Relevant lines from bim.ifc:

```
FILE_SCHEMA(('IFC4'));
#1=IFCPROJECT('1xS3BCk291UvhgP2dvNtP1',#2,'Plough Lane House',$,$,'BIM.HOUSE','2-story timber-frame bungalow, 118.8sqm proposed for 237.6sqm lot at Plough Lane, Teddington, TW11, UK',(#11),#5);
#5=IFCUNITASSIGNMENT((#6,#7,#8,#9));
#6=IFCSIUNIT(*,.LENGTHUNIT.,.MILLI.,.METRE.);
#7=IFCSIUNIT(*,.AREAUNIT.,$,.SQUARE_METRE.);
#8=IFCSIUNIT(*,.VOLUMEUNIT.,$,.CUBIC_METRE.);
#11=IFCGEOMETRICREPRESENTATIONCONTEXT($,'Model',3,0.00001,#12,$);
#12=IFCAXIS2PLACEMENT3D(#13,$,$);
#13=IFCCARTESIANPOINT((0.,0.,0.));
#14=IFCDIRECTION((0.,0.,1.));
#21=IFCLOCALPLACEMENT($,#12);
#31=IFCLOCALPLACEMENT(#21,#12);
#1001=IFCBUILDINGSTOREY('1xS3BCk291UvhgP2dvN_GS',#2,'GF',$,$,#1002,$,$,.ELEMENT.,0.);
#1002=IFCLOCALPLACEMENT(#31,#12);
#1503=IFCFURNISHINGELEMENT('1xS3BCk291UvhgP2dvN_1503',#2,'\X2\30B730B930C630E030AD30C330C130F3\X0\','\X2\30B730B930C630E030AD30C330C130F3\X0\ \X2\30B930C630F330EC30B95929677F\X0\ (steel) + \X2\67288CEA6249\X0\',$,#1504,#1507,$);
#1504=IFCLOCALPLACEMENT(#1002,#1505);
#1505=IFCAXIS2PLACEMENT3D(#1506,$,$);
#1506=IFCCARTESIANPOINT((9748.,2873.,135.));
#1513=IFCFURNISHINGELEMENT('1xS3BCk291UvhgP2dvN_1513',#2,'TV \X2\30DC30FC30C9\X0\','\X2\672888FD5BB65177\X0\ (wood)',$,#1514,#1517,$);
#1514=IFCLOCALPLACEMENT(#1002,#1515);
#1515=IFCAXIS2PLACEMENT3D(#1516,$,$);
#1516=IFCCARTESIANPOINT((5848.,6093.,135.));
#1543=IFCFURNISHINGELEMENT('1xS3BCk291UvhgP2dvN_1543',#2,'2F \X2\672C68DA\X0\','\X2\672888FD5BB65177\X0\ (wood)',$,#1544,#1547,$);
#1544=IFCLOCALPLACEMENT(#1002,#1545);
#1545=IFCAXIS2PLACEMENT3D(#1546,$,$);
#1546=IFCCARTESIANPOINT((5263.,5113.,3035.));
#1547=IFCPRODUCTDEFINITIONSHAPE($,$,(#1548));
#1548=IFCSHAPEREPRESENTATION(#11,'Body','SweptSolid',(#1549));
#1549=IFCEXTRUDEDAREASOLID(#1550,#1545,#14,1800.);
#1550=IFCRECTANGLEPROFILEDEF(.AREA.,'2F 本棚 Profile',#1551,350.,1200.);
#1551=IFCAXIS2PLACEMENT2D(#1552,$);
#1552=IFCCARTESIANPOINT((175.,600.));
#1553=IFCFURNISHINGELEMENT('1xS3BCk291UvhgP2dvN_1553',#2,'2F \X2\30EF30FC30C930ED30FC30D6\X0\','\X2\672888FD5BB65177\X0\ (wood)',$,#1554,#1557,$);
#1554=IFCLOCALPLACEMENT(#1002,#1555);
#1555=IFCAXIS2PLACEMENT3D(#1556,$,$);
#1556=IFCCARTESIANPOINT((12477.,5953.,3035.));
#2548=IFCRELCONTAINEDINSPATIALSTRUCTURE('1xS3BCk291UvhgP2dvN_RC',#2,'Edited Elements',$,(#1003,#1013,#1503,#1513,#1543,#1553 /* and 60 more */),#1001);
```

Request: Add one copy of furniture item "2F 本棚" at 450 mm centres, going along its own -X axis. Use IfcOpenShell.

```python
import ifcopenshell
import ifcopenshell.api.geometry
import ifcopenshell.api.root
import ifcopenshell.util.element
import ifcopenshell.util.placement

model = ifcopenshell.open("bim.ifc")


def reuse_history(source, copy):
    """copy_class also copies each property set's owner history, people and application; keep the originals."""
    for rel in copy.IsDefinedBy:
        if rel.is_a("IfcRelDefinesByProperties") and (history := rel.RelatingPropertyDefinition.OwnerHistory):
            rel.RelatingPropertyDefinition.OwnerHistory = source.OwnerHistory
            ifcopenshell.util.element.remove_deep2(model, history)


source = model.by_id(1543)
base = ifcopenshell.util.placement.get_local_placement(source.ObjectPlacement)
step = -base[:3, 0] * 450.0

for i in range(1, 2):
    copy = ifcopenshell.api.root.copy_class(model, product=source)
    copy.Representation = ifcopenshell.util.element.copy_deep(
        model, source.Representation, exclude=["IfcGeometricRepresentationContext", "IfcRepresentationMap"]
    )
    reuse_history(source, copy)
    matrix = base.copy()
    matrix[:3, 3] += i * step
    print("added at", matrix[:3, 3].round(3) + 0.0)
    ifcopenshell.api.geometry.edit_object_placement(model, product=copy, matrix=matrix, is_si=False)

model.write("bim_updated.ifc")
```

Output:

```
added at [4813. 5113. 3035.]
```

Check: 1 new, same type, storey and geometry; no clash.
